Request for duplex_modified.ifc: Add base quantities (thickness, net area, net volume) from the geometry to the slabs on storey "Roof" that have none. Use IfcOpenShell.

First a look at what the model holds.

```python
import ifcopenshell
import ifcopenshell.util.element
import ifcopenshell.util.unit

model = ifcopenshell.open("duplex_modified.ifc")
print(model.schema)
for unit_type in ("LENGTHUNIT", "AREAUNIT", "VOLUMEUNIT"):
    print(unit_type, ifcopenshell.util.unit.calculate_unit_scale(model, unit_type))
storey = next(s for s in model.by_type("IfcBuildingStorey") if s.Name == "Roof")
slabs = [e for e in ifcopenshell.util.element.get_decomposition(storey) if e.is_a("IfcSlab")]
for e in sorted(slabs, key=lambda e: e.id()):
    print(e.id(), e.is_a(), e.Name, list(ifcopenshell.util.element.get_psets(e, qtos_only=True)), sep=" | ")
```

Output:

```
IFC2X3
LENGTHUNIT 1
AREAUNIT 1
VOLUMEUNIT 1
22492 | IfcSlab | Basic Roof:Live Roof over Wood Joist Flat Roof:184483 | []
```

```python
import ifcopenshell
import ifcopenshell.api.pset
import ifcopenshell.geom
import ifcopenshell.util.element
import ifcopenshell.util.shape
import ifcopenshell.util.unit

model = ifcopenshell.open("duplex_modified.ifc")
unit_scale = ifcopenshell.util.unit.calculate_unit_scale(model)
area_scale = ifcopenshell.util.unit.calculate_unit_scale(model, "AREAUNIT")
volume_scale = ifcopenshell.util.unit.calculate_unit_scale(model, "VOLUMEUNIT")
settings = ifcopenshell.geom.settings()

storey = next(s for s in model.by_type("IfcBuildingStorey") if s.Name == "Roof")
slabs = [e for e in ifcopenshell.util.element.get_decomposition(storey) if e.is_a("IfcSlab")]

for e in sorted(slabs, key=lambda e: e.id()):
    if ifcopenshell.util.element.get_psets(e, qtos_only=True, should_inherit=False):
        continue
    # Geometry comes back in metres, in the element's own axes.
    shape = ifcopenshell.geom.create_shape(settings, e)
    values = {
        "Width": ifcopenshell.util.shape.get_z(shape.geometry) / unit_scale,
        "NetArea": ifcopenshell.util.shape.get_footprint_area(shape.geometry) / area_scale,
        "NetVolume": ifcopenshell.util.shape.get_volume(shape.geometry) / volume_scale,
    }
    qto = ifcopenshell.api.pset.add_qto(model, product=e, name="BaseQuantities")
    ifcopenshell.api.pset.edit_qto(model, qto=qto, properties=values)
    print(e.id(), {k: round(v, 3) for k, v in values.items()})

model.write("duplex_modified_edited.ifc")
```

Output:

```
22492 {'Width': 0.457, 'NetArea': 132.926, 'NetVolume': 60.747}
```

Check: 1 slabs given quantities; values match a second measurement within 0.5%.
